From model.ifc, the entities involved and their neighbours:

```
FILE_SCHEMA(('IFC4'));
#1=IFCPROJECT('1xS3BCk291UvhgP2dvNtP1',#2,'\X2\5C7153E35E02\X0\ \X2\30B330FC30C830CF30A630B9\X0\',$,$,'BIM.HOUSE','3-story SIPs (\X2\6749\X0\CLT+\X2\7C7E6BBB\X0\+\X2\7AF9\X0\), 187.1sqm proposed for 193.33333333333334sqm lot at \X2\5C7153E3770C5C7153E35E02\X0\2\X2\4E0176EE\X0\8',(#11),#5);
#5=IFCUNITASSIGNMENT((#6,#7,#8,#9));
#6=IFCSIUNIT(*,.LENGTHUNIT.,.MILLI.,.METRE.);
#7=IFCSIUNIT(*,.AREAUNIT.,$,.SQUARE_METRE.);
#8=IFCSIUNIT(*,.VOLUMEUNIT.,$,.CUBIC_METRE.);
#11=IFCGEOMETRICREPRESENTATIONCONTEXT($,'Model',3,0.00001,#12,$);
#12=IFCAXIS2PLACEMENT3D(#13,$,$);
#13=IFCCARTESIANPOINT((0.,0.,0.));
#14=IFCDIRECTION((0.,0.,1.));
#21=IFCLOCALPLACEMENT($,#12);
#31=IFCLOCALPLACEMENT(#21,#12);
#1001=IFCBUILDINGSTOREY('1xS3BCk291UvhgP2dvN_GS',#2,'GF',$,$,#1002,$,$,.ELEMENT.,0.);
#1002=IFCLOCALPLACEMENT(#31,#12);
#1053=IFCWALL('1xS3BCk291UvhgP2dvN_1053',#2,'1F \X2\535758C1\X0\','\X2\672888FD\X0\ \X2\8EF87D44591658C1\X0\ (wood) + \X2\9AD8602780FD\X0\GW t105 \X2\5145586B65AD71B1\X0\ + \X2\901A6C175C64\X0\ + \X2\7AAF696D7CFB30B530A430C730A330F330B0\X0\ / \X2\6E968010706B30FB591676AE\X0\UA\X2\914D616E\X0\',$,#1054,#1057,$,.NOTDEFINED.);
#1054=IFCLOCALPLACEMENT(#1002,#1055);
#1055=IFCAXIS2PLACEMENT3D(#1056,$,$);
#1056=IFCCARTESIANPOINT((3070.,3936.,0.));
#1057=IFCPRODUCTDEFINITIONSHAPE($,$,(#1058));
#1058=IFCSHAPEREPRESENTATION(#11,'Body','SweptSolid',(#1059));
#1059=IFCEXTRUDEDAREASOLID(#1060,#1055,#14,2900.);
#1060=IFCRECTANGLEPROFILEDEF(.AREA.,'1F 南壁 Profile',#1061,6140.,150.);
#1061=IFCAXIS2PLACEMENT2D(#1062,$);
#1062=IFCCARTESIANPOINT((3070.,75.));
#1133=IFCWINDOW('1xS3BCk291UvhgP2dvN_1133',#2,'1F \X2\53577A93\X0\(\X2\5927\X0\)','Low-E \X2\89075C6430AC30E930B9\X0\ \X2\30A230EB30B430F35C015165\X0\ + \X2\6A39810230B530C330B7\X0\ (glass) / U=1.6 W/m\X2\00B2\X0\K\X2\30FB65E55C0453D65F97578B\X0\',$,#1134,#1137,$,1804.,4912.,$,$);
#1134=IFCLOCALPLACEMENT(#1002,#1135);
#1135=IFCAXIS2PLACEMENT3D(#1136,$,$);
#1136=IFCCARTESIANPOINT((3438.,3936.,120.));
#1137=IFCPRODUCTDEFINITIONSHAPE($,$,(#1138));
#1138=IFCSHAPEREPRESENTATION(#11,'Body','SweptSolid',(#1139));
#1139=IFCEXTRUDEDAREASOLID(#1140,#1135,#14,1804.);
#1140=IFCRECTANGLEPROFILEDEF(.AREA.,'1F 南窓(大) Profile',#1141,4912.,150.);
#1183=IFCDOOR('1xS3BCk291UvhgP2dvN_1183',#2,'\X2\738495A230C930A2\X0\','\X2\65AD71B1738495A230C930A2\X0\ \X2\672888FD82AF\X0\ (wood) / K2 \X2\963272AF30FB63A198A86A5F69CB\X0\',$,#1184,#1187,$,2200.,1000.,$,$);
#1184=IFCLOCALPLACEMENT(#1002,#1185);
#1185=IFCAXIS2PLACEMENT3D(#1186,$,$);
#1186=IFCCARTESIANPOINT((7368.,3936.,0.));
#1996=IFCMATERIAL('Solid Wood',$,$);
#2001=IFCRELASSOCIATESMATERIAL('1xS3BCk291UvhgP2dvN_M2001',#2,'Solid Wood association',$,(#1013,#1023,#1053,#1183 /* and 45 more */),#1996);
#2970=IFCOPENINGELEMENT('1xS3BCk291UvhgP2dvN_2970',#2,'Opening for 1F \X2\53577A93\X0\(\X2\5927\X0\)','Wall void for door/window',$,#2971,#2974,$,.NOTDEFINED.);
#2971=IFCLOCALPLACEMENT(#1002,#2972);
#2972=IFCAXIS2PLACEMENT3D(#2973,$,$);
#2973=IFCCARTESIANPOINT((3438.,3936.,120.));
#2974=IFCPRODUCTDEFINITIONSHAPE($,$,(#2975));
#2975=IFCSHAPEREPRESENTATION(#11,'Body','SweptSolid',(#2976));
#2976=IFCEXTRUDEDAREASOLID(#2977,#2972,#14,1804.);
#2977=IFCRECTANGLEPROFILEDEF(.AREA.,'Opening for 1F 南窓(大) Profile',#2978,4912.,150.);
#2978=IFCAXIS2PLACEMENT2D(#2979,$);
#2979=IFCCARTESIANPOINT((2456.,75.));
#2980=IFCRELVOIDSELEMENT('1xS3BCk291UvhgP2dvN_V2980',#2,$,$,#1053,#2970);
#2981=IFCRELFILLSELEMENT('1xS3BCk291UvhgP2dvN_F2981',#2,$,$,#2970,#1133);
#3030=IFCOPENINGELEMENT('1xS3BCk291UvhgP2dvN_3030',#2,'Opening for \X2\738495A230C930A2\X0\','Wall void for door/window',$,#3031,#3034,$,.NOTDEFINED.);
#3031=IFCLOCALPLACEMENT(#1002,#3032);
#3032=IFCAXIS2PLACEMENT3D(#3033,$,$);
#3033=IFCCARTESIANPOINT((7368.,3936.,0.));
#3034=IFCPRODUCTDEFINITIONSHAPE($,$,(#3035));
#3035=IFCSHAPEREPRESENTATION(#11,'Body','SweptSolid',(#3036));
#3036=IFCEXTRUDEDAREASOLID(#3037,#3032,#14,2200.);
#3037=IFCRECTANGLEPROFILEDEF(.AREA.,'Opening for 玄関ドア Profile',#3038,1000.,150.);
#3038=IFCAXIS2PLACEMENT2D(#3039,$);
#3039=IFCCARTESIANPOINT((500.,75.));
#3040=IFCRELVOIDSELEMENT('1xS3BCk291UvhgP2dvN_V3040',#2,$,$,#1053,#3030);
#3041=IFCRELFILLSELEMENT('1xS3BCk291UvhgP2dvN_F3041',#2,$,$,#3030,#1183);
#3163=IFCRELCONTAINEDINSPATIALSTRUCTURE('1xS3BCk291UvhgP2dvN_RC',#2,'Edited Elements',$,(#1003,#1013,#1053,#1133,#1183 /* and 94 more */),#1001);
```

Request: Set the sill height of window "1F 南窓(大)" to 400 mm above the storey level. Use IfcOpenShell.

```python
import numpy as np
import ifcopenshell
import ifcopenshell.api.geometry
import ifcopenshell.geom
import ifcopenshell.util.element
import ifcopenshell.util.placement
import ifcopenshell.util.shape
import ifcopenshell.util.unit

model = ifcopenshell.open("model.ifc")
unit_scale = ifcopenshell.util.unit.calculate_unit_scale(model)

window = model.by_guid("1xS3BCk291UvhgP2dvN_1133")
opening = window.FillsVoids[0].RelatingOpeningElement
storey = ifcopenshell.util.element.get_container(window, ifc_class="IfcBuildingStorey")
level = ifcopenshell.util.placement.get_local_placement(storey.ObjectPlacement)[2, 3]

# The opening's origin need not be at the sill, so measure its lowest point.
shape = ifcopenshell.geom.create_shape(ifcopenshell.geom.settings(), opening)
bottom = ifcopenshell.util.shape.get_shape_bottom_elevation(shape, shape.geometry) / unit_scale
dz = level + 400.0 - bottom

shift = np.array([0.0, 0.0, dz])
# The window is not placed relative to its opening, so move both.
for product in (opening, window):
    matrix = ifcopenshell.util.placement.get_local_placement(product.ObjectPlacement)
    matrix[:3, 3] += shift
    ifcopenshell.api.geometry.edit_object_placement(model, product=product, matrix=matrix, is_si=False)

print(f"moved by {dz * unit_scale:+.3f} m")

model.write("model_updated.ifc")
```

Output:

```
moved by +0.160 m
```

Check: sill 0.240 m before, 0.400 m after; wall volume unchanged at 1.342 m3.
